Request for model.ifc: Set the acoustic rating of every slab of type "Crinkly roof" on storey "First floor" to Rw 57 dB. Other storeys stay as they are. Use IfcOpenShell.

First a look at what the model holds.

```python
import ifcopenshell
import ifcopenshell.util.element

model = ifcopenshell.open("model.ifc")
print(model.schema)
storey = next(s for s in model.by_type("IfcBuildingStorey") if s.Name == "First floor")
slabs = [e for e in ifcopenshell.util.element.get_decomposition(storey) if e.is_a("IfcSlab")]
seen = {}
for e in slabs:
    element_type = ifcopenshell.util.element.get_type(e)
    key = (element_type.Name if element_type != e and element_type else None, ifcopenshell.util.element.get_pset(e, "Pset_SlabCommon", "AcousticRating"))
    seen[key] = seen.get(key, 0) + 1
for (name, value), count in sorted(seen.items(), key=str):
    print(count, "x", name, "|", value)
```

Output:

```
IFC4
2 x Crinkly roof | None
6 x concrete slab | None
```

```python
import ifcopenshell
import ifcopenshell.api.pset
import ifcopenshell.util.element

model = ifcopenshell.open("model.ifc")

storey = next(s for s in model.by_type("IfcBuildingStorey") if s.Name == "First floor")
slabs = [e for e in ifcopenshell.util.element.get_decomposition(storey) if e.is_a("IfcSlab")]

count = 0
for e in slabs:
    element_type = ifcopenshell.util.element.get_type(e)
    if element_type in (None, e) or element_type.Name != "Crinkly roof":
        continue
    # add_pset returns the element's existing set when there is one.
    pset = ifcopenshell.api.pset.add_pset(model, product=e, name="Pset_SlabCommon")
    ifcopenshell.api.pset.edit_pset(model, pset=pset, properties={"AcousticRating": "Rw 57 dB"})
    count += 1

print(count, "slabs updated")

model.write("model_v2.ifc")
```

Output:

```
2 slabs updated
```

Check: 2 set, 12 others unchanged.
